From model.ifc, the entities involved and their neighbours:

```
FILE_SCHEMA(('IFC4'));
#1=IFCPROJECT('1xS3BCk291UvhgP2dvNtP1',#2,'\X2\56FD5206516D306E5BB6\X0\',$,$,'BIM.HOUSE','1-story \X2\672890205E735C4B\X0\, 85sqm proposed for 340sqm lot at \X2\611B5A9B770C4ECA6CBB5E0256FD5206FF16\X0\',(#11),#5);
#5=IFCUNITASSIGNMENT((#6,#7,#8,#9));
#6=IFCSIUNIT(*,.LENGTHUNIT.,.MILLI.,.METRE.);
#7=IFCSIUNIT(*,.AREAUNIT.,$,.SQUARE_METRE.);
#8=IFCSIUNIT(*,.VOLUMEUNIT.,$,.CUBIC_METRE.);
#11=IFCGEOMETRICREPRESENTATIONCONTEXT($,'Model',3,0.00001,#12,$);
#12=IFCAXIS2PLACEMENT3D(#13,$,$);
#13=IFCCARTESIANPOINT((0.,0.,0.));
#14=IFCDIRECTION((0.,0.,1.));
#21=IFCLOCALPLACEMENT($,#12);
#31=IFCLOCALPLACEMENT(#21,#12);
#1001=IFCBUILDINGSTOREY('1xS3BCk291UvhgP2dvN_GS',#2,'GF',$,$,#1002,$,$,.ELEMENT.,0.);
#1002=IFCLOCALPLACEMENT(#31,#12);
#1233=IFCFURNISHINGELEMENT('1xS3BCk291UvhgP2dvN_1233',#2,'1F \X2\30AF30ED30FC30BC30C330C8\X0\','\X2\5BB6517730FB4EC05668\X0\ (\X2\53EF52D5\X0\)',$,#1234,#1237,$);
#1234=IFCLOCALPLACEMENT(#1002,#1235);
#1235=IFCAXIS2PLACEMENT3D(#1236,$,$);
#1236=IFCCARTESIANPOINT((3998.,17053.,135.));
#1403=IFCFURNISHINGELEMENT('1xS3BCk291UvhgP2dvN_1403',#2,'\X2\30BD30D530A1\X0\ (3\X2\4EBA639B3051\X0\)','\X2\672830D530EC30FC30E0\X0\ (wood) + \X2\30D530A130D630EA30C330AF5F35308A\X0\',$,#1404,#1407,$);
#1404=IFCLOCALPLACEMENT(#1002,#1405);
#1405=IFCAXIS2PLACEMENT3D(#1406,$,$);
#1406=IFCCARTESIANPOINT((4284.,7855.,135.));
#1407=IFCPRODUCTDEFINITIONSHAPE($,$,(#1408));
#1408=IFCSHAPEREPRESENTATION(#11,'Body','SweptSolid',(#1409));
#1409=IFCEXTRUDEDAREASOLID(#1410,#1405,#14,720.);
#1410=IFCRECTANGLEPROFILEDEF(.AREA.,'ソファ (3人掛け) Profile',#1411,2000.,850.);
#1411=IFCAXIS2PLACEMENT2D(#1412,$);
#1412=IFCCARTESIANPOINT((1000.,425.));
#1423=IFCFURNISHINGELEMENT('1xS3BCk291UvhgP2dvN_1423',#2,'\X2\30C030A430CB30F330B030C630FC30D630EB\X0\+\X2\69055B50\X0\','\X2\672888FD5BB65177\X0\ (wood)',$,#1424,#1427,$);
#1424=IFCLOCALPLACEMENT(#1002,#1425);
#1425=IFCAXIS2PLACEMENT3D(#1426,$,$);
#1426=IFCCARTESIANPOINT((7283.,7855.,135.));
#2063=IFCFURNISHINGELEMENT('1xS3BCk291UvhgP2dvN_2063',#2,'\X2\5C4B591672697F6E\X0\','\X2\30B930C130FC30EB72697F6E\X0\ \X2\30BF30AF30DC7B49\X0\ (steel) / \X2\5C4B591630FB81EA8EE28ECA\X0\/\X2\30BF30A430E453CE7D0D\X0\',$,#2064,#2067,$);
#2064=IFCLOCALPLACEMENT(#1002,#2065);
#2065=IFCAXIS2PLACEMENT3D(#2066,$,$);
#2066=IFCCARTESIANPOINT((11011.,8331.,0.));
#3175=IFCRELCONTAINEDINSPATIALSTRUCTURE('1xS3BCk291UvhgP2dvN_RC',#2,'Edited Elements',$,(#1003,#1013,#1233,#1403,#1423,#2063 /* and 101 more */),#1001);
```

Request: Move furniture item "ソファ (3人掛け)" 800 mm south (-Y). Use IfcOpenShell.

```python
import ifcopenshell
import ifcopenshell.api.geometry
import ifcopenshell.util.placement
import ifcopenshell.util.unit

model = ifcopenshell.open("model.ifc")
unit_scale = ifcopenshell.util.unit.calculate_unit_scale(model)

item = model.by_guid("1xS3BCk291UvhgP2dvN_1403")
matrix = ifcopenshell.util.placement.get_local_placement(item.ObjectPlacement)
matrix[1, 3] -= 0.8 / unit_scale
ifcopenshell.api.geometry.edit_object_placement(model, product=item, matrix=matrix, is_si=False)

print(ifcopenshell.util.placement.get_local_placement(item.ObjectPlacement).round(3) + 0.0)

model.write("model-out.ifc")
```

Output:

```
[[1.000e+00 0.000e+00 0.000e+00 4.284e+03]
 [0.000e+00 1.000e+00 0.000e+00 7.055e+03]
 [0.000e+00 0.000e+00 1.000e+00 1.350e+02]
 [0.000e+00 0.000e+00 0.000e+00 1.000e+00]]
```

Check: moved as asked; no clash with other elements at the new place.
